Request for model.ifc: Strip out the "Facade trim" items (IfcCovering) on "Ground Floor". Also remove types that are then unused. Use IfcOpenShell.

First a look at what the model holds.

```python
import ifcopenshell
import ifcopenshell.util.element

model = ifcopenshell.open("model.ifc")
print(model.schema)
storey = next(s for s in model.by_type("IfcBuildingStorey") if s.Name == "Ground Floor")
coverings = [e for e in ifcopenshell.util.element.get_decomposition(storey) if e.is_a("IfcCovering")]
seen = {}
for e in coverings:
    element_type = ifcopenshell.util.element.get_type(e)
    name = element_type.Name if element_type not in (None, e) else None
    seen[name] = seen.get(name, 0) + 1
for name, count in sorted(seen.items(), key=str):
    print(count, "x", name)
```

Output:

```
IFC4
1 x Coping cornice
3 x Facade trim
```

```python
import ifcopenshell
import ifcopenshell.api.root
import ifcopenshell.util.element

model = ifcopenshell.open("model.ifc")

storey = next(s for s in model.by_type("IfcBuildingStorey") if s.Name == "Ground Floor")
coverings = [e for e in ifcopenshell.util.element.get_decomposition(storey) if e.is_a("IfcCovering")]
targets = [e for e in coverings if (t := ifcopenshell.util.element.get_type(e)) not in (None, e) and t.Name == "Facade trim"]
types = {ifcopenshell.util.element.get_type(e) for e in targets} - {None, *targets}

for e in targets:
    ifcopenshell.api.root.remove_product(model, product=e)
print(len(targets), "removed")

unused = [t for t in types if not ifcopenshell.util.element.get_types(t)]
for t in unused:
    ifcopenshell.api.root.remove_product(model, product=t)
print(len(unused), "unused types removed")

model.write("model_rev.ifc")
```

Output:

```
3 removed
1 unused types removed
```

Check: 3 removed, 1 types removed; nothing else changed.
